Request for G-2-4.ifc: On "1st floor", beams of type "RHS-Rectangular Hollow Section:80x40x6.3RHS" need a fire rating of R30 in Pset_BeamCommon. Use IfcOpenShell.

First a look at what the model holds.

```python
import ifcopenshell
import ifcopenshell.util.element

model = ifcopenshell.open("G-2-4.ifc")
print(model.schema)
storey = next(s for s in model.by_type("IfcBuildingStorey") if s.Name == "1st floor")
beams = [e for e in ifcopenshell.util.element.get_decomposition(storey) if e.is_a("IfcBeam")]
seen = {}
for e in beams:
    element_type = ifcopenshell.util.element.get_type(e)
    key = (element_type.Name if element_type != e and element_type else None, ifcopenshell.util.element.get_pset(e, "Pset_BeamCommon", "FireRating"))
    seen[key] = seen.get(key, 0) + 1
for (name, value), count in sorted(seen.items(), key=str):
    print(count, "x", name, "|", value)
```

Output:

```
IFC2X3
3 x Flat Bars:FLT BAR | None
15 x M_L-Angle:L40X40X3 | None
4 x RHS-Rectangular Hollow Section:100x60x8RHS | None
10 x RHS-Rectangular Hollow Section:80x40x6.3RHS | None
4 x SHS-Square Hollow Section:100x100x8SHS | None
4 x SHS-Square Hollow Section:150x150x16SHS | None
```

```python
import ifcopenshell
import ifcopenshell.api.pset
import ifcopenshell.util.element

model = ifcopenshell.open("G-2-4.ifc")

storey = next(s for s in model.by_type("IfcBuildingStorey") if s.Name == "1st floor")
beams = [e for e in ifcopenshell.util.element.get_decomposition(storey) if e.is_a("IfcBeam")]

count = 0
for e in beams:
    element_type = ifcopenshell.util.element.get_type(e)
    if element_type in (None, e) or element_type.Name != "RHS-Rectangular Hollow Section:80x40x6.3RHS":
        continue
    # add_pset returns the element's existing set when there is one.
    pset = ifcopenshell.api.pset.add_pset(model, product=e, name="Pset_BeamCommon")
    ifcopenshell.api.pset.edit_pset(model, pset=pset, properties={"FireRating": "R30"})
    count += 1

print(count, "beams updated")

model.write("G-2-4_updated.ifc")
```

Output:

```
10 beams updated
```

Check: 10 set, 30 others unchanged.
